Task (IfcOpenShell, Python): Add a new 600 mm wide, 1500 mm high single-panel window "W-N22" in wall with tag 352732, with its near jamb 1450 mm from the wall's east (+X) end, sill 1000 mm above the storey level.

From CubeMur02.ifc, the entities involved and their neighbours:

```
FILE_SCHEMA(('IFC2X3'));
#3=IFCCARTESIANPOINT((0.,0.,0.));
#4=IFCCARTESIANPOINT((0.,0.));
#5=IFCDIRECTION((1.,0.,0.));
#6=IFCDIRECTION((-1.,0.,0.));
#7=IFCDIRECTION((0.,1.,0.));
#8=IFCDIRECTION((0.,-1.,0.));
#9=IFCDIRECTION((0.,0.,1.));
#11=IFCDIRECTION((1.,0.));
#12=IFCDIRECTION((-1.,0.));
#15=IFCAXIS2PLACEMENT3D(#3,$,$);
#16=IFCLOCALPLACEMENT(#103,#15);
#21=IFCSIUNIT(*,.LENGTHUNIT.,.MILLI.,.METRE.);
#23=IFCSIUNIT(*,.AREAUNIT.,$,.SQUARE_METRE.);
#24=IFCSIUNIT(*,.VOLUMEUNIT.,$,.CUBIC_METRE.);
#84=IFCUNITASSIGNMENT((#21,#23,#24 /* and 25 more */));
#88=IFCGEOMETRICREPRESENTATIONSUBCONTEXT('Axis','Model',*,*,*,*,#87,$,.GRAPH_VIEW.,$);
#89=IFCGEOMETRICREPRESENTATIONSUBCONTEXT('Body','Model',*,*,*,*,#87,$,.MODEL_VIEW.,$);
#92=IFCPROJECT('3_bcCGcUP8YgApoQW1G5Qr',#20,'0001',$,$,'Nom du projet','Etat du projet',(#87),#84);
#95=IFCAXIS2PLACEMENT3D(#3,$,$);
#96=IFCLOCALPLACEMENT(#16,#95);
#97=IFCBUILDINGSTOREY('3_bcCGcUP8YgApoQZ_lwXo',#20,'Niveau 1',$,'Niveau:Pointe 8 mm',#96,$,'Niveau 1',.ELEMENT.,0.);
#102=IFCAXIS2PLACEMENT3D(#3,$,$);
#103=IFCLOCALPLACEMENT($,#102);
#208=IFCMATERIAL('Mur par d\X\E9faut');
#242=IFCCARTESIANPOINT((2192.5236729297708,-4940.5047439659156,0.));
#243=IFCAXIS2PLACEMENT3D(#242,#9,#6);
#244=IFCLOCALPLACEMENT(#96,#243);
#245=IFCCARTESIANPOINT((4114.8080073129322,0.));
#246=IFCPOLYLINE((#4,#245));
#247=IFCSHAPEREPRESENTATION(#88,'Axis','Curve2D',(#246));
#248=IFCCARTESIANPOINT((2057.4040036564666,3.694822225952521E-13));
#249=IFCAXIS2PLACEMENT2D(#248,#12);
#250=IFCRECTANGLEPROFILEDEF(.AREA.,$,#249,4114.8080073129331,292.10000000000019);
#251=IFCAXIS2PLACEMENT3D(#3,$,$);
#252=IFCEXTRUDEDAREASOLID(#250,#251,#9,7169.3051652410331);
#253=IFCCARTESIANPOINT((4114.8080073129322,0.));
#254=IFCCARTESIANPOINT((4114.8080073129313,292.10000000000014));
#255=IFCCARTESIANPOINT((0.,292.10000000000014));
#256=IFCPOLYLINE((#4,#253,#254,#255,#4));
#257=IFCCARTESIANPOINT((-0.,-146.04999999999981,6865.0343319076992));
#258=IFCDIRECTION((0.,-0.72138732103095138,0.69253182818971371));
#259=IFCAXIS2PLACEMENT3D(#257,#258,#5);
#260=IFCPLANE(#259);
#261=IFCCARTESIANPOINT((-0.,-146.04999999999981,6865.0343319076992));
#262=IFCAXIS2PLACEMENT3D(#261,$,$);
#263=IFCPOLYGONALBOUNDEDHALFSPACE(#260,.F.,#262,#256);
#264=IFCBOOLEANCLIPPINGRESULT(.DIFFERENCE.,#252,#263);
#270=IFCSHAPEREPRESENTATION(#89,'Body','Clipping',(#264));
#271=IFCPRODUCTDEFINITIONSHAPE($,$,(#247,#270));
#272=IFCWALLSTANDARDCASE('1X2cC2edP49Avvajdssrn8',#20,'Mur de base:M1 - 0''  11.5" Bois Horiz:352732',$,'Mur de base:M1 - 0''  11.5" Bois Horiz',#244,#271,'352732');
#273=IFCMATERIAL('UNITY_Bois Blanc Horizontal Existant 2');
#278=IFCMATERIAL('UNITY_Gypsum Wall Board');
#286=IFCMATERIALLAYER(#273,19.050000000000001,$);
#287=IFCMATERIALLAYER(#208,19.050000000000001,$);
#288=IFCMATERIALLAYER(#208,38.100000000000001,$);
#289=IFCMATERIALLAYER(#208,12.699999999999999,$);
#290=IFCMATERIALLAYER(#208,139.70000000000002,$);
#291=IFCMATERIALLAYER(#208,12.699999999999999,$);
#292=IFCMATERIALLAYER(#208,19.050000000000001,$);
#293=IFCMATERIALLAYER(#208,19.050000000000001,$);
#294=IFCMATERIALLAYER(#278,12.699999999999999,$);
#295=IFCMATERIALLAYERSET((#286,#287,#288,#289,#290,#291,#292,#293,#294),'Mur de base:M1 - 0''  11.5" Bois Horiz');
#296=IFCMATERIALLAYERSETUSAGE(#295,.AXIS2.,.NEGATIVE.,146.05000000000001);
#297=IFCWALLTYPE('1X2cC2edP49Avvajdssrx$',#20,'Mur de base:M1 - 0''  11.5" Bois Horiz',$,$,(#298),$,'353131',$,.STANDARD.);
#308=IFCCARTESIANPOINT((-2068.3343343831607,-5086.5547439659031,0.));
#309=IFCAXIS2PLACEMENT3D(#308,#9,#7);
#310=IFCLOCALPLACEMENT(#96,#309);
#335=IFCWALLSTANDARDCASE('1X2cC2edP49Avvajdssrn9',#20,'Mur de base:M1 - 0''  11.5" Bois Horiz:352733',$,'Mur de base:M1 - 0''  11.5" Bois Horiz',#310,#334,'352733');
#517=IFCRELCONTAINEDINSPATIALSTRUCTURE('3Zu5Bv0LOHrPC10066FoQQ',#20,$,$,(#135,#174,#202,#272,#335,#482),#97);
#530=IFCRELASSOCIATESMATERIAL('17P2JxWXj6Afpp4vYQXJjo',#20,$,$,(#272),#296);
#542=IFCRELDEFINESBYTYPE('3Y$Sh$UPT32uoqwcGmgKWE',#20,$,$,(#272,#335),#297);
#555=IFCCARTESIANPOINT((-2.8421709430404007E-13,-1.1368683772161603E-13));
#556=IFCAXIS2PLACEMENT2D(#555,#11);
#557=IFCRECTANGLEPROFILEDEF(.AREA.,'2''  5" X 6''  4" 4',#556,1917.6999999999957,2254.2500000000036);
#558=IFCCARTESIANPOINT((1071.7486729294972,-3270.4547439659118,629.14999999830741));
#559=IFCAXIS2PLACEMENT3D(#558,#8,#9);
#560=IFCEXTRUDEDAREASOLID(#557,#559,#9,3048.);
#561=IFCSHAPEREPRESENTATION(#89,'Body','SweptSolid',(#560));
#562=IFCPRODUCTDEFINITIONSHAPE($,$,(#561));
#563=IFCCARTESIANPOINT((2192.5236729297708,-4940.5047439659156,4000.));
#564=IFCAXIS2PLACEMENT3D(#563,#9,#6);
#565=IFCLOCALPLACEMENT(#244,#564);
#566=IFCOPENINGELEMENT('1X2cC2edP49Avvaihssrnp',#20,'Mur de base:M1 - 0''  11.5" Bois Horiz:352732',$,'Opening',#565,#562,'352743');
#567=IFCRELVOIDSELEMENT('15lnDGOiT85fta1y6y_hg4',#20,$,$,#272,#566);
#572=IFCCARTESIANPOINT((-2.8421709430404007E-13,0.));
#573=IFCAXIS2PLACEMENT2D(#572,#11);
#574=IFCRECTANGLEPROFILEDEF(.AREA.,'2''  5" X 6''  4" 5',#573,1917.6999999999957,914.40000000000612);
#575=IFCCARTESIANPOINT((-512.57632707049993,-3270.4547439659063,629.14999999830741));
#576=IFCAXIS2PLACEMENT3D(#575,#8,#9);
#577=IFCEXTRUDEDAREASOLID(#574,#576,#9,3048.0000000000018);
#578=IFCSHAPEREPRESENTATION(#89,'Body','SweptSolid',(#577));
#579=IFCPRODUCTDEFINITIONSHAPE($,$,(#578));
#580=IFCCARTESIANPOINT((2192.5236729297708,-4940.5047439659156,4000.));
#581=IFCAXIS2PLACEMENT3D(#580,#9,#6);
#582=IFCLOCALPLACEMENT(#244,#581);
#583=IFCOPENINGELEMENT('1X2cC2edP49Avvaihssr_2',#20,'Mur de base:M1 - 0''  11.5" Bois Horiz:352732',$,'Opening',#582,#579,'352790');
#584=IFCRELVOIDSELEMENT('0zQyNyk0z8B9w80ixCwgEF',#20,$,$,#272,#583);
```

```python
import numpy as np
import ifcopenshell
import ifcopenshell.api.feature
import ifcopenshell.api.geometry
import ifcopenshell.api.root
import ifcopenshell.api.spatial
import ifcopenshell.api.type
import ifcopenshell.geom
import ifcopenshell.util.element
import ifcopenshell.util.placement
import ifcopenshell.util.representation
import ifcopenshell.util.shape
import ifcopenshell.util.unit

model = ifcopenshell.open("CubeMur02.ifc")
unit_scale = ifcopenshell.util.unit.calculate_unit_scale(model)
settings = ifcopenshell.geom.settings()


def volume(element):
    """Net volume in cubic metres, openings subtracted."""
    shape = ifcopenshell.geom.create_shape(settings, element)
    return ifcopenshell.util.shape.get_volume(shape.geometry)


wall = model.by_guid("1X2cC2edP49Avvajdssrn8")
storey = ifcopenshell.util.element.get_container(wall, ifc_class="IfcBuildingStorey")
context = ifcopenshell.util.representation.get_context(model, "Model", "Body", "MODEL_VIEW")
before = volume(wall)

width, height, from_end, sill = 0.6, 1.5, 1.45, 1  # metres

# The wall runs along its own X axis, and the end named is its -X end.
wall_shape = ifcopenshell.geom.create_shape(settings, wall)
x, y, z = ifcopenshell.util.shape.get_vertices(wall_shape.geometry).T
start = x.min() + from_end
face, thickness = float(y.min()), float(y.max() - y.min())
wall_matrix = ifcopenshell.util.placement.get_local_placement(wall.ObjectPlacement)
level = ifcopenshell.util.placement.get_local_placement(storey.ObjectPlacement)[2, 3]


def in_wall(x, y):
    """Placement at x, y metres in the wall's axes, at sill height."""
    matrix = wall_matrix.copy()
    matrix[:, 3] = wall_matrix @ np.array([x / unit_scale, y / unit_scale, 0.0, 1.0])
    matrix[2, 3] = level + sill / unit_scale
    return matrix


# Opening: a box that overshoots both wall faces by 50 mm.
opening = ifcopenshell.api.root.create_entity(model, ifc_class="IfcOpeningElement")
box = ifcopenshell.api.geometry.add_wall_representation(
    model, context=context, length=width, height=height, thickness=thickness + 0.1
)
ifcopenshell.api.geometry.assign_representation(model, product=opening, representation=box)
ifcopenshell.api.geometry.edit_object_placement(model, product=opening, matrix=in_wall(start, face - 0.05), is_si=False)
ifcopenshell.api.feature.add_feature(model, feature=opening, element=wall)

window = ifcopenshell.api.root.create_entity(model, ifc_class="IfcWindow", name="W-N22")
window.OverallWidth, window.OverallHeight = width / unit_scale, height / unit_scale
body = ifcopenshell.api.geometry.add_window_representation(
    model,
    context=context,
    overall_width=window.OverallWidth,
    overall_height=window.OverallHeight,
    partition_type="SINGLE_PANEL",
)
ifcopenshell.api.geometry.assign_representation(model, product=window, representation=body)
ifcopenshell.api.spatial.assign_container(model, products=[window], relating_structure=storey)
fills = ifcopenshell.api.feature.add_filling(model, opening=opening, element=window)
fills.OwnerHistory = window.OwnerHistory  # required in IFC2X3

# IFC2X3 keeps the operation on the window style.
style = ifcopenshell.api.root.create_entity(model, ifc_class="IfcWindowStyle", name="W-N22")
style.OperationType, style.ConstructionType = "SINGLE_PANEL", "NOTDEFINED"
style.ParameterTakesPrecedence = style.Sizeable = False
ifcopenshell.api.type.assign_type(model, related_objects=[window], relating_type=style)

# Centre the window in the wall's thickness.
ifcopenshell.api.geometry.edit_object_placement(model, product=window, matrix=in_wall(start, face), is_si=False)
window_shape = ifcopenshell.geom.create_shape(settings, window)
depth = ifcopenshell.util.shape.get_vertices(window_shape.geometry)[:, 1]
offset = face + thickness / 2 - (depth.min() + depth.max()) / 2
ifcopenshell.api.geometry.edit_object_placement(model, product=window, matrix=in_wall(start, offset), is_si=False)

after = volume(wall)

print(f"wall volume {before:.3f} -> {after:.3f} m3")

model.write("CubeMur02_v2.ifc")
```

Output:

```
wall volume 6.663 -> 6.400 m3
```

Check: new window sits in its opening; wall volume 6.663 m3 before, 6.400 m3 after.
